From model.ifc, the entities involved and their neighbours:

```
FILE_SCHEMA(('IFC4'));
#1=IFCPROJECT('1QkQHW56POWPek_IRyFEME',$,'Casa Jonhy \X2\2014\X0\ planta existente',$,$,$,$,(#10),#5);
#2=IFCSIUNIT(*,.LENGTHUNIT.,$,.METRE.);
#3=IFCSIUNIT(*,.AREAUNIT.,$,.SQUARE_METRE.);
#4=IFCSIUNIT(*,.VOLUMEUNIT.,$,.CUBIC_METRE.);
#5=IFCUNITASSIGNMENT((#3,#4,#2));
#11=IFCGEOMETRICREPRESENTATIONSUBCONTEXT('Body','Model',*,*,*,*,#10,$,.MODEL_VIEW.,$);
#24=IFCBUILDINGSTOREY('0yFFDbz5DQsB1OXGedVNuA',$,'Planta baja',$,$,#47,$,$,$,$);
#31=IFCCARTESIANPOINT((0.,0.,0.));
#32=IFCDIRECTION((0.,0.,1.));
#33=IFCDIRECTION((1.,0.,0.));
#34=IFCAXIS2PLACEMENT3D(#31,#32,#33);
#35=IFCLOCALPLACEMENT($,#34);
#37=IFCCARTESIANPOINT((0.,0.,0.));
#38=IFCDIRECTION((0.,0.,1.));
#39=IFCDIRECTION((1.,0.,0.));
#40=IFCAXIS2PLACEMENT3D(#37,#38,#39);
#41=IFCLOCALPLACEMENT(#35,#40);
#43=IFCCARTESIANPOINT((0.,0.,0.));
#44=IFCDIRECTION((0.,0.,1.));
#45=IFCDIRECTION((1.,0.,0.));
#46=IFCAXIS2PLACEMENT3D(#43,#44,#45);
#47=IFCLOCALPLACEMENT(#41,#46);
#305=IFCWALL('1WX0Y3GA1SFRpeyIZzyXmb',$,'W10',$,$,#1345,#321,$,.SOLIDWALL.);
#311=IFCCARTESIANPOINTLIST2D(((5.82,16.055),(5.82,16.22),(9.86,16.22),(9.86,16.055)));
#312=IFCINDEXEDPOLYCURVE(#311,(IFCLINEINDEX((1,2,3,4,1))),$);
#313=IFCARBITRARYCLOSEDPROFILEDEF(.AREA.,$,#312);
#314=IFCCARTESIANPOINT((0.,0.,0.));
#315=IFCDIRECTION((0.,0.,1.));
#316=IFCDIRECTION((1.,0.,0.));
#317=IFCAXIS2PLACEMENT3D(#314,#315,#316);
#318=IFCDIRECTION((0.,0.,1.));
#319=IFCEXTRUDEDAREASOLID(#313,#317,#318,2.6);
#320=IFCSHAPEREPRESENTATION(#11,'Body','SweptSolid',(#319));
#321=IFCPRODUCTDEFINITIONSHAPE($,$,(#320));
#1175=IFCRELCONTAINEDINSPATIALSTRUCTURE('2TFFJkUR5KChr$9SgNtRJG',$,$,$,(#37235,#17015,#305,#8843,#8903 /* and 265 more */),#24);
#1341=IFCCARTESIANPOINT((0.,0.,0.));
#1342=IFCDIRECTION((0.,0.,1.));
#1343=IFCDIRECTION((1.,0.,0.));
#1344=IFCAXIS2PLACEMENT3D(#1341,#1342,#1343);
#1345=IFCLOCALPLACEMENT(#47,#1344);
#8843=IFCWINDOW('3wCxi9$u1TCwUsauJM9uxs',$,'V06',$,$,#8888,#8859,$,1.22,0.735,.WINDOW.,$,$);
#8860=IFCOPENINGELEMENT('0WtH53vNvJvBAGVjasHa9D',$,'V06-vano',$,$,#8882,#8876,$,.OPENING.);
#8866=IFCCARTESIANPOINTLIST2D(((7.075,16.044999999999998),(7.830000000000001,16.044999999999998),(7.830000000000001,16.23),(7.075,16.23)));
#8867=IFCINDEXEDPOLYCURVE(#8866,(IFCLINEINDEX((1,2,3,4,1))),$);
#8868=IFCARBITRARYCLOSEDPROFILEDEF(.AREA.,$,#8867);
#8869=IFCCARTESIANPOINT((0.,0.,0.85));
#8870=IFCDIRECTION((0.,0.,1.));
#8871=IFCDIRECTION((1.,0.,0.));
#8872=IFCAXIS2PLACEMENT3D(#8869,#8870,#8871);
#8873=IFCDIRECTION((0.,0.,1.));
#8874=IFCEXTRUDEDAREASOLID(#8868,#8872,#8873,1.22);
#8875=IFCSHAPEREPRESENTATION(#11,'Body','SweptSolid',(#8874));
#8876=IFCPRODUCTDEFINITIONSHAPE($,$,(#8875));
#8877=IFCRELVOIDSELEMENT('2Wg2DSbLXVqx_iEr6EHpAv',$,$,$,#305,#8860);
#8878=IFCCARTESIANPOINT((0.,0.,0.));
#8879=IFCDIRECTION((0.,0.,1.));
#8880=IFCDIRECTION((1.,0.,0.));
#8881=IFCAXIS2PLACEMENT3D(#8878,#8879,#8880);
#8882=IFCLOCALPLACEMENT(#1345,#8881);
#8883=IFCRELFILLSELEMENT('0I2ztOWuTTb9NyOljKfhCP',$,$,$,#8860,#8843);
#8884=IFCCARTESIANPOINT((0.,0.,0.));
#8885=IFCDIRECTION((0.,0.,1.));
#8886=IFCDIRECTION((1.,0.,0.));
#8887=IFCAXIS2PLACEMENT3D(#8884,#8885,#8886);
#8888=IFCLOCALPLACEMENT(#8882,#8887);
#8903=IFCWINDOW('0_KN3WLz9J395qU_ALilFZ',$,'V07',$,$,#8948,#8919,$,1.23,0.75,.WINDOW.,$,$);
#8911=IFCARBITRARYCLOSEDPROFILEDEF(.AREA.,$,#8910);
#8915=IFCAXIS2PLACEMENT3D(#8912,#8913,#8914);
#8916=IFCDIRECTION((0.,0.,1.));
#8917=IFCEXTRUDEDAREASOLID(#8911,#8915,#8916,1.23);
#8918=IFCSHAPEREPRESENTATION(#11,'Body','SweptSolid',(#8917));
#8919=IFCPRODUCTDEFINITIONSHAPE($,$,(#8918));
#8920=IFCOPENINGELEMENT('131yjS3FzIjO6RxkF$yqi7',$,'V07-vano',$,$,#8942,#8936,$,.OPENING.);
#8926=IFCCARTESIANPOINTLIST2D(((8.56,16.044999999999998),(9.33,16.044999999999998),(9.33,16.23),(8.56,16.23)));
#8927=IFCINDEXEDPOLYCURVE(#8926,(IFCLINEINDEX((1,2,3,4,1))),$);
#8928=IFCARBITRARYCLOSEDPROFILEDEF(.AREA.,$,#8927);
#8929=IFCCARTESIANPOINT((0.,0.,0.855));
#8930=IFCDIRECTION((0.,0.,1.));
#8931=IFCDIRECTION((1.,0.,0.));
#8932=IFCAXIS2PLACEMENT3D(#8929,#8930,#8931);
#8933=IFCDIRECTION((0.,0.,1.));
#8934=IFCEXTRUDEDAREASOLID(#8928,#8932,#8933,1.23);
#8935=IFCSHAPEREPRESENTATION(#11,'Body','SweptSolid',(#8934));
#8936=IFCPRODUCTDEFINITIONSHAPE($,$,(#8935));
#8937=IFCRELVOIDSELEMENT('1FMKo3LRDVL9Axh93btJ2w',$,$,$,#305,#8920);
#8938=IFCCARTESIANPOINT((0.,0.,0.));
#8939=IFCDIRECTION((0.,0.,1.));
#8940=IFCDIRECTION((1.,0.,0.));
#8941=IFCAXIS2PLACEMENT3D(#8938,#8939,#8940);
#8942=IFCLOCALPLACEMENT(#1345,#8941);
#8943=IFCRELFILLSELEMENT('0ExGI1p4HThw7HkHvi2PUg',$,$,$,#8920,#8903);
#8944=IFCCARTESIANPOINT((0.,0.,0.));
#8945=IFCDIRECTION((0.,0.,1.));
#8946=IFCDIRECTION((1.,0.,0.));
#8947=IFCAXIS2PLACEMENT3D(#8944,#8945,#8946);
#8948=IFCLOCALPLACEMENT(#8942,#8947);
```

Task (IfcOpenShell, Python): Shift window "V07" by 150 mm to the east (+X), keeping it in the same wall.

```python
import ifcopenshell
import ifcopenshell.api.geometry
import ifcopenshell.util.placement
import ifcopenshell.util.unit

model = ifcopenshell.open("model.ifc")
unit_scale = ifcopenshell.util.unit.calculate_unit_scale(model)

window = model.by_guid("0_KN3WLz9J395qU_ALilFZ")
opening = window.FillsVoids[0].RelatingOpeningElement
wall = opening.VoidsElements[0].RelatingBuildingElement

wall_matrix = ifcopenshell.util.placement.get_local_placement(wall.ObjectPlacement)
shift = wall_matrix[:3, 0] * 0.15 / unit_scale
before = ifcopenshell.util.placement.get_local_placement(window.ObjectPlacement)[:3, 3].copy()

# The window is placed relative to its opening, so it follows when the opening moves.
matrix = ifcopenshell.util.placement.get_local_placement(opening.ObjectPlacement)
matrix[:3, 3] += shift
ifcopenshell.api.geometry.edit_object_placement(
    model, product=opening, matrix=matrix, is_si=False, should_transform_children=True
)

after = ifcopenshell.util.placement.get_local_placement(window.ObjectPlacement)[:3, 3]
print("window moved by", (after - before).round(3) + 0.0)

model.write("model_edited.ifc")
```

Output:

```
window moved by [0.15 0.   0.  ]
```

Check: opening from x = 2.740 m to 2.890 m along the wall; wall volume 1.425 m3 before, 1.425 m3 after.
